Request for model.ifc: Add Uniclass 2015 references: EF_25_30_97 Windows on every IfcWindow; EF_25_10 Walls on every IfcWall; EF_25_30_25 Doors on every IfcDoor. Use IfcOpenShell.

First a look at what the model holds.

```python
import ifcopenshell

model = ifcopenshell.open("model.ifc")
print(model.schema)
print("classifications:", [c.Name for c in model.by_type("IfcClassification")])
for ifc_class in ("IfcDoor", "IfcRoof", "IfcStair", "IfcWall", "IfcWindow"):
    print(ifc_class, len(model.by_type(ifc_class)))
```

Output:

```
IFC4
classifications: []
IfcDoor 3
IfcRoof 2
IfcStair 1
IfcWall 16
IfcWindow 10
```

```python
import ifcopenshell
import ifcopenshell.api.classification

model = ifcopenshell.open("model.ifc")

system = ifcopenshell.api.classification.add_classification(model, classification="Uniclass 2015")

codes = {
    "IfcWindow": ("EF_25_30_97", "Windows"),
    "IfcWall": ("EF_25_10", "Walls"),
    "IfcDoor": ("EF_25_30_25", "Doors"),
}
for ifc_class, (code, name) in codes.items():
    products = model.by_type(ifc_class)
    ifcopenshell.api.classification.add_reference(
        model, products=products, classification=system, identification=code, name=name
    )
    print(code, len(products))

model.write("model-out.ifc")
```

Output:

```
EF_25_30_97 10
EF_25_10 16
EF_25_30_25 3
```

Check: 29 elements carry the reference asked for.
